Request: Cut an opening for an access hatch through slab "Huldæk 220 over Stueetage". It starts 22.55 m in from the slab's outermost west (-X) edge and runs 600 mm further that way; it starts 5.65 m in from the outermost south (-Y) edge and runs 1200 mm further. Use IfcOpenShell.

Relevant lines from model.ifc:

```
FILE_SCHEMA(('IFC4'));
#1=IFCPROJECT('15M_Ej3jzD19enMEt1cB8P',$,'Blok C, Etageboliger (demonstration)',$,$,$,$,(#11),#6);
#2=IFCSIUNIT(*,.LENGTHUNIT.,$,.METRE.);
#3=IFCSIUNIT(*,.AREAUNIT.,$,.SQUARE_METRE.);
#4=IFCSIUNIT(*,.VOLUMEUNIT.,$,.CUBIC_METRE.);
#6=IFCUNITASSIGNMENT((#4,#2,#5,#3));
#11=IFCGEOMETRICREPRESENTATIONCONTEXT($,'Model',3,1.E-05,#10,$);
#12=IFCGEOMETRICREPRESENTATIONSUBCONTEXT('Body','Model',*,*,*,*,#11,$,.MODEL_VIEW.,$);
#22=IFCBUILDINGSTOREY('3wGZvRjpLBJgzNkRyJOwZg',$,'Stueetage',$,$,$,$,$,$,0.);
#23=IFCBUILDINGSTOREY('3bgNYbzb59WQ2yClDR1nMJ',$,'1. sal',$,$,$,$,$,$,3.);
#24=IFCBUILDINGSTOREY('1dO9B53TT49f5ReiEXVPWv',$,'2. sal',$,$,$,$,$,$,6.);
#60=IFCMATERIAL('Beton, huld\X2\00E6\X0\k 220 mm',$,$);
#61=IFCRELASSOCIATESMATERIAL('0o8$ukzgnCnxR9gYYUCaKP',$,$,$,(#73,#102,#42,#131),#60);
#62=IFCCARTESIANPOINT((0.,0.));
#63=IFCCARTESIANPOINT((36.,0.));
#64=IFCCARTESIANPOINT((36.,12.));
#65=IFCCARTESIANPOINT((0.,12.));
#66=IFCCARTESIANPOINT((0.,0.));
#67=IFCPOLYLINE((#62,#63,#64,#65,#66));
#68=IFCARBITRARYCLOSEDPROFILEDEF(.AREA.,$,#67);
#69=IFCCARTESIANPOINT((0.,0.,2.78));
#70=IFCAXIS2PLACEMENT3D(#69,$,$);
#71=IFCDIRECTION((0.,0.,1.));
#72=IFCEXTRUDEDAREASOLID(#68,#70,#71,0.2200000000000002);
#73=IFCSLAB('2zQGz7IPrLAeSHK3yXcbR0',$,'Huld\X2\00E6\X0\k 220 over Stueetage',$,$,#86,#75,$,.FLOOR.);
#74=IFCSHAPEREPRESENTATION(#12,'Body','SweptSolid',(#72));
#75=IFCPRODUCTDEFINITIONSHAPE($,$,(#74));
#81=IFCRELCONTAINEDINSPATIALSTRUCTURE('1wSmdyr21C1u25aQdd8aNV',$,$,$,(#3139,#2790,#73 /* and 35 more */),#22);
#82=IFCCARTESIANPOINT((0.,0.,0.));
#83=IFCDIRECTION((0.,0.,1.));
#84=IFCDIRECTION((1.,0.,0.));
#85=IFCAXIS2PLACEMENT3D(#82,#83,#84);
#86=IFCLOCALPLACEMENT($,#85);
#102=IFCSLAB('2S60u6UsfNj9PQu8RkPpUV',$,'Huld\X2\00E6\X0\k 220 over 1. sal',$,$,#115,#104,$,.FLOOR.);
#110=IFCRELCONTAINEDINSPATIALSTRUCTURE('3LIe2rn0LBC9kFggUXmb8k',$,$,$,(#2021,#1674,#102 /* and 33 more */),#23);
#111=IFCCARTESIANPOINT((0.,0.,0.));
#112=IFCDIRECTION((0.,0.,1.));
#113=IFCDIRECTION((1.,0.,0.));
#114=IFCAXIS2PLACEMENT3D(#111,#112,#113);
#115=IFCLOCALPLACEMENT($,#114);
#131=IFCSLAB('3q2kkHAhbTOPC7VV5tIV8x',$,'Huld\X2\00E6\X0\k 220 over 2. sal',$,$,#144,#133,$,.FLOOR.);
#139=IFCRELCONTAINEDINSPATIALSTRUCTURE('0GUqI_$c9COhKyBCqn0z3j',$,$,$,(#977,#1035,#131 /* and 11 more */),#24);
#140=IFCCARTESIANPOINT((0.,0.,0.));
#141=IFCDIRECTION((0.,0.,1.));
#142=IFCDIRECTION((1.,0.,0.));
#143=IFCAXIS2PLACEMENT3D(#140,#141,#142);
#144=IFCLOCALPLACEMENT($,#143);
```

```python
import numpy as np
import ifcopenshell
import ifcopenshell.api.feature
import ifcopenshell.api.geometry
import ifcopenshell.api.root
import ifcopenshell.geom
import ifcopenshell.util.placement
import ifcopenshell.util.representation
import ifcopenshell.util.shape
import ifcopenshell.util.unit

model = ifcopenshell.open("model.ifc")
unit_scale = ifcopenshell.util.unit.calculate_unit_scale(model)
settings = ifcopenshell.geom.settings()


def volume(element):
    """Net volume in cubic metres, openings subtracted."""
    shape = ifcopenshell.geom.create_shape(settings, element)
    return ifcopenshell.util.shape.get_volume(shape.geometry)


slab = model.by_guid("2zQGz7IPrLAeSHK3yXcbR0")
before = volume(slab)

# Extent in the slab's own axes, in metres. The edges named are its -X and -Y sides.
slab_shape = ifcopenshell.geom.create_shape(settings, slab)
vertices = ifcopenshell.util.shape.get_vertices(slab_shape.geometry)
x_min, y_min, bottom = vertices.min(axis=0)
top = vertices[:, 2].max()

opening = ifcopenshell.api.root.create_entity(model, ifc_class="IfcOpeningElement", name="Access hatch opening", predefined_type="OPENING")
context = ifcopenshell.util.representation.get_context(model, "Model", "Body", "MODEL_VIEW")
width, depth = 0.6, 1.2
outline = [(0.0, 0.0), (width, 0.0), (width, depth), (0.0, depth), (0.0, 0.0)]
# Overshoot both faces by 50 mm so the cut is clean.
shape = ifcopenshell.api.geometry.add_slab_representation(
    model, context=context, depth=top - bottom + 0.1, polyline=outline
)
ifcopenshell.api.geometry.assign_representation(model, product=opening, representation=shape)

matrix = ifcopenshell.util.placement.get_local_placement(slab.ObjectPlacement)
matrix[:, 3] = matrix @ np.append(np.array([x_min + 22.55, y_min + 5.65, bottom - 0.05]) / unit_scale, 1.0)
ifcopenshell.api.geometry.edit_object_placement(model, product=opening, matrix=matrix, is_si=False)
ifcopenshell.api.feature.add_feature(model, feature=opening, element=slab)

after = volume(slab)

print(f"slab volume {before:.3f} -> {after:.3f} m3")

model.write("model_v2.ifc")
```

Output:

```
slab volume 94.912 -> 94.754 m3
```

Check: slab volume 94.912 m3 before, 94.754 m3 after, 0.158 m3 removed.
